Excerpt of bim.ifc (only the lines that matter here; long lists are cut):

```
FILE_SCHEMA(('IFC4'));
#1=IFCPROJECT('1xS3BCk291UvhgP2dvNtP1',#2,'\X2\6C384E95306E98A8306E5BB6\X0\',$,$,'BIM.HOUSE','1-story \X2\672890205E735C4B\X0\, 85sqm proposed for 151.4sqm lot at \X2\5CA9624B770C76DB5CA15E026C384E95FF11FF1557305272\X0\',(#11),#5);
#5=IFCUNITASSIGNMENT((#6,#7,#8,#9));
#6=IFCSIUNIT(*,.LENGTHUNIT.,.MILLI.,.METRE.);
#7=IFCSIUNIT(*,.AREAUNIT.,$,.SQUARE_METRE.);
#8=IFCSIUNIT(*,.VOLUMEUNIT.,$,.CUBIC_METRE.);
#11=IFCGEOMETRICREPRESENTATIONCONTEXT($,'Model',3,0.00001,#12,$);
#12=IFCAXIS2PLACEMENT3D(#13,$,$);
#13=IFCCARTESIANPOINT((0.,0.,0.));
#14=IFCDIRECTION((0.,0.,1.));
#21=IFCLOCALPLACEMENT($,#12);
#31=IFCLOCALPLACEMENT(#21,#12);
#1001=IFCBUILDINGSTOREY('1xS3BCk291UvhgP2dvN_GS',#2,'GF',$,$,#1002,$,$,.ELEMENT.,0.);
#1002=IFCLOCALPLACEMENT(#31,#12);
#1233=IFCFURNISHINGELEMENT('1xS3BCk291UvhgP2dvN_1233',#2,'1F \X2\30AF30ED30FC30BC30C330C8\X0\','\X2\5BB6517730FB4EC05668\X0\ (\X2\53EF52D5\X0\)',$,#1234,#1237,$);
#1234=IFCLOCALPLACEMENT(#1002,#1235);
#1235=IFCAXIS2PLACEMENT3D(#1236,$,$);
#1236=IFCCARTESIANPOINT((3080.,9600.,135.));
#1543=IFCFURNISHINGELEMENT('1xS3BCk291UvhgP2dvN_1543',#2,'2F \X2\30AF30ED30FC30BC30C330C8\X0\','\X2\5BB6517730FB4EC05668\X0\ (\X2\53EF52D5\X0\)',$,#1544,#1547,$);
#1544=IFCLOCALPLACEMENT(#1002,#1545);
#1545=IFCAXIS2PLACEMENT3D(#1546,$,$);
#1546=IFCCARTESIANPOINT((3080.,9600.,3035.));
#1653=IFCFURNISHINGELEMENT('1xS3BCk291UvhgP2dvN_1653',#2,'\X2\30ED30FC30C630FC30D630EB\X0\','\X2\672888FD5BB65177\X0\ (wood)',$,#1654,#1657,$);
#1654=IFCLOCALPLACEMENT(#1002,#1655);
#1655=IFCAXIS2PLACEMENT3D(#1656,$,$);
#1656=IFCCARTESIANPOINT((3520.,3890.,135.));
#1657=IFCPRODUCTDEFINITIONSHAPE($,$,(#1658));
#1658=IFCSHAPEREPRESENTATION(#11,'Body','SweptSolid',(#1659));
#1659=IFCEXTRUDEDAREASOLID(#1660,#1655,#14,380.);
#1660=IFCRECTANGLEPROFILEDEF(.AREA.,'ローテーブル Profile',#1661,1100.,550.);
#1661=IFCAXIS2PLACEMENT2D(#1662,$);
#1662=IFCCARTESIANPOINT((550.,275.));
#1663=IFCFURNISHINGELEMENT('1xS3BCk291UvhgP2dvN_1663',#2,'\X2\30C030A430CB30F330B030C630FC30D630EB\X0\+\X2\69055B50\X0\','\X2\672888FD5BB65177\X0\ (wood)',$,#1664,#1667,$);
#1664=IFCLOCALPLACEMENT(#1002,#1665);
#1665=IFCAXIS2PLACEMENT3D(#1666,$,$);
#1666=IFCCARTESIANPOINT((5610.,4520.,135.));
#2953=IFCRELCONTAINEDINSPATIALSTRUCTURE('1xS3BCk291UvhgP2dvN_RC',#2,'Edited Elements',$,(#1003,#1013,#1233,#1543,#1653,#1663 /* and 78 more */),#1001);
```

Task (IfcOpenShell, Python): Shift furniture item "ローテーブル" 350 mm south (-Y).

```python
import ifcopenshell
import ifcopenshell.api.geometry
import ifcopenshell.util.placement
import ifcopenshell.util.unit

model = ifcopenshell.open("bim.ifc")
unit_scale = ifcopenshell.util.unit.calculate_unit_scale(model)

item = model.by_id(1653)
matrix = ifcopenshell.util.placement.get_local_placement(item.ObjectPlacement)
matrix[1, 3] -= 0.35 / unit_scale
ifcopenshell.api.geometry.edit_object_placement(model, product=item, matrix=matrix, is_si=False)

print(ifcopenshell.util.placement.get_local_placement(item.ObjectPlacement).round(3) + 0.0)

model.write("bim_updated.ifc")
```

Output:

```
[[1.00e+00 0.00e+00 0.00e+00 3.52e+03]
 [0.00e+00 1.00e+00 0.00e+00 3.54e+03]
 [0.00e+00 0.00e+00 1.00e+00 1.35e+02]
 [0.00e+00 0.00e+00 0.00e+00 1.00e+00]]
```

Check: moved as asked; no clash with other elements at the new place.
